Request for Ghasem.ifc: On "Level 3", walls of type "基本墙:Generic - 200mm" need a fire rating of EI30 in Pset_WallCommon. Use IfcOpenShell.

First a look at what the model holds.

```python
import ifcopenshell
import ifcopenshell.util.element

model = ifcopenshell.open("Ghasem.ifc")
print(model.schema)
storey = next(s for s in model.by_type("IfcBuildingStorey") if s.Name == "Level 3")
walls = [e for e in ifcopenshell.util.element.get_decomposition(storey) if e.is_a("IfcWall")]
seen = {}
for e in walls:
    element_type = ifcopenshell.util.element.get_type(e)
    key = (element_type.Name if element_type != e and element_type else None, ifcopenshell.util.element.get_pset(e, "Pset_WallCommon", "FireRating"))
    seen[key] = seen.get(key, 0) + 1
for (name, value), count in sorted(seen.items(), key=str):
    print(count, "x", name, "|", value)
```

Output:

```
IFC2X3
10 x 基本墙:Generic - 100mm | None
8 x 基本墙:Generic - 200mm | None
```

```python
import ifcopenshell
import ifcopenshell.api.pset
import ifcopenshell.util.element

model = ifcopenshell.open("Ghasem.ifc")

storey = next(s for s in model.by_type("IfcBuildingStorey") if s.Name == "Level 3")
walls = [e for e in ifcopenshell.util.element.get_decomposition(storey) if e.is_a("IfcWall")]

count = 0
for e in walls:
    element_type = ifcopenshell.util.element.get_type(e)
    if element_type in (None, e) or element_type.Name != "基本墙:Generic - 200mm":
        continue
    # add_pset returns the element's existing set when there is one.
    pset = ifcopenshell.api.pset.add_pset(model, product=e, name="Pset_WallCommon")
    ifcopenshell.api.pset.edit_pset(model, pset=pset, properties={"FireRating": "EI30"})
    count += 1

print(count, "walls updated")

model.write("Ghasem_updated.ifc")
```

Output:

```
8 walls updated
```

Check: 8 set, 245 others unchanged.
